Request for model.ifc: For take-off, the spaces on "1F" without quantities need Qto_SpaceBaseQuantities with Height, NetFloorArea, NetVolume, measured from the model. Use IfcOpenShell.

First a look at what the model holds.

```python
import ifcopenshell
import ifcopenshell.util.element
import ifcopenshell.util.unit

model = ifcopenshell.open("model.ifc")
print(model.schema)
for unit_type in ("LENGTHUNIT", "AREAUNIT", "VOLUMEUNIT"):
    print(unit_type, ifcopenshell.util.unit.calculate_unit_scale(model, unit_type))
storey = next(s for s in model.by_type("IfcBuildingStorey") if s.Name == "1F")
spaces = [e for e in ifcopenshell.util.element.get_decomposition(storey) if e.is_a("IfcSpace")]
for e in sorted(spaces, key=lambda e: e.id()):
    print(e.id(), e.is_a(), e.Name, list(ifcopenshell.util.element.get_psets(e, qtos_only=True)), sep=" | ")
```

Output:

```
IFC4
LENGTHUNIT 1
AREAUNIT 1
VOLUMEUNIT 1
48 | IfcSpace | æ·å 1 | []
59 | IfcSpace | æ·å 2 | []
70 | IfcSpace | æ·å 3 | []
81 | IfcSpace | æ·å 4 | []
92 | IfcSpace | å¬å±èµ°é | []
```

```python
import ifcopenshell
import ifcopenshell.api.pset
import ifcopenshell.geom
import ifcopenshell.util.element
import ifcopenshell.util.shape
import ifcopenshell.util.unit

model = ifcopenshell.open("model.ifc")
unit_scale = ifcopenshell.util.unit.calculate_unit_scale(model)
area_scale = ifcopenshell.util.unit.calculate_unit_scale(model, "AREAUNIT")
volume_scale = ifcopenshell.util.unit.calculate_unit_scale(model, "VOLUMEUNIT")
settings = ifcopenshell.geom.settings()

storey = next(s for s in model.by_type("IfcBuildingStorey") if s.Name == "1F")
spaces = [e for e in ifcopenshell.util.element.get_decomposition(storey) if e.is_a("IfcSpace")]

for e in sorted(spaces, key=lambda e: e.id()):
    if ifcopenshell.util.element.get_psets(e, qtos_only=True, should_inherit=False):
        continue
    # Geometry comes back in metres, in the element's own axes.
    shape = ifcopenshell.geom.create_shape(settings, e)
    values = {
        "Height": ifcopenshell.util.shape.get_z(shape.geometry) / unit_scale,
        "NetFloorArea": ifcopenshell.util.shape.get_footprint_area(shape.geometry) / area_scale,
        "NetVolume": ifcopenshell.util.shape.get_volume(shape.geometry) / volume_scale,
    }
    qto = ifcopenshell.api.pset.add_qto(model, product=e, name="Qto_SpaceBaseQuantities")
    ifcopenshell.api.pset.edit_qto(model, qto=qto, properties=values)
    print(e.id(), {k: round(v, 3) for k, v in values.items()})

model.write("model-out.ifc")
```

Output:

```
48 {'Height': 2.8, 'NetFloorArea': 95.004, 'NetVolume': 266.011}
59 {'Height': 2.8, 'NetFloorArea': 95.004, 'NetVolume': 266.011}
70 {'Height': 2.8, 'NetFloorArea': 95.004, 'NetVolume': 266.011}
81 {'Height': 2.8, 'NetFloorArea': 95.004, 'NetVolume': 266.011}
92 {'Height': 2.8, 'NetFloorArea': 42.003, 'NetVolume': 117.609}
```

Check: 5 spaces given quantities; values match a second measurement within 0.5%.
